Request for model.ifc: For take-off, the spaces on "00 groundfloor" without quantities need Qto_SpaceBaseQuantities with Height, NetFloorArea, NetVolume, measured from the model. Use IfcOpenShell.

First a look at what the model holds.

```python
import ifcopenshell
import ifcopenshell.util.element
import ifcopenshell.util.unit

model = ifcopenshell.open("model.ifc")
print(model.schema)
for unit_type in ("LENGTHUNIT", "AREAUNIT", "VOLUMEUNIT"):
    print(unit_type, ifcopenshell.util.unit.calculate_unit_scale(model, unit_type))
storey = next(s for s in model.by_type("IfcBuildingStorey") if s.Name == "00 groundfloor")
spaces = [e for e in ifcopenshell.util.element.get_decomposition(storey) if e.is_a("IfcSpace")]
for e in sorted(spaces, key=lambda e: e.id()):
    print(e.id(), e.is_a(), e.Name, list(ifcopenshell.util.element.get_psets(e, qtos_only=True)), sep=" | ")
```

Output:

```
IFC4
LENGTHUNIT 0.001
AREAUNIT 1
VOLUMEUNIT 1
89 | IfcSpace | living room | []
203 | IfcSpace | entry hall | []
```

```python
import ifcopenshell
import ifcopenshell.api.pset
import ifcopenshell.geom
import ifcopenshell.util.element
import ifcopenshell.util.shape
import ifcopenshell.util.unit

model = ifcopenshell.open("model.ifc")
unit_scale = ifcopenshell.util.unit.calculate_unit_scale(model)
area_scale = ifcopenshell.util.unit.calculate_unit_scale(model, "AREAUNIT")
volume_scale = ifcopenshell.util.unit.calculate_unit_scale(model, "VOLUMEUNIT")
settings = ifcopenshell.geom.settings()

storey = next(s for s in model.by_type("IfcBuildingStorey") if s.Name == "00 groundfloor")
spaces = [e for e in ifcopenshell.util.element.get_decomposition(storey) if e.is_a("IfcSpace")]

for e in sorted(spaces, key=lambda e: e.id()):
    if ifcopenshell.util.element.get_psets(e, qtos_only=True, should_inherit=False):
        continue
    # Geometry comes back in metres, in the element's own axes.
    shape = ifcopenshell.geom.create_shape(settings, e)
    values = {
        "Height": ifcopenshell.util.shape.get_z(shape.geometry) / unit_scale,
        "NetFloorArea": ifcopenshell.util.shape.get_footprint_area(shape.geometry) / area_scale,
        "NetVolume": ifcopenshell.util.shape.get_volume(shape.geometry) / volume_scale,
    }
    qto = ifcopenshell.api.pset.add_qto(model, product=e, name="Qto_SpaceBaseQuantities")
    ifcopenshell.api.pset.edit_qto(model, qto=qto, properties=values)
    print(e.id(), {k: round(v, 3) for k, v in values.items()})

model.write("model-out.ifc")
```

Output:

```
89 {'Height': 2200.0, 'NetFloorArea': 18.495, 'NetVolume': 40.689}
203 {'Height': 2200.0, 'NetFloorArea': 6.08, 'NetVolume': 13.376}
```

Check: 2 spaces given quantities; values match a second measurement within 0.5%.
